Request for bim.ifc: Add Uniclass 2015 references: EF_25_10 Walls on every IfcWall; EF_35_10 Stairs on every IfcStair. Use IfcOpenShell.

First a look at what the model holds.

```python
import ifcopenshell

model = ifcopenshell.open("bim.ifc")
print(model.schema)
print("classifications:", [c.Name for c in model.by_type("IfcClassification")])
for ifc_class in ("IfcDoor", "IfcRoof", "IfcStair", "IfcWall", "IfcWindow"):
    print(ifc_class, len(model.by_type(ifc_class)))
```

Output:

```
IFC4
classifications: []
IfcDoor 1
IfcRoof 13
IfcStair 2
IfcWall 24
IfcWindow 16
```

```python
import ifcopenshell
import ifcopenshell.api.classification

model = ifcopenshell.open("bim.ifc")

system = ifcopenshell.api.classification.add_classification(model, classification="Uniclass 2015")

codes = {
    "IfcWall": ("EF_25_10", "Walls"),
    "IfcStair": ("EF_35_10", "Stairs"),
}
for ifc_class, (code, name) in codes.items():
    products = model.by_type(ifc_class)
    ifcopenshell.api.classification.add_reference(
        model, products=products, classification=system, identification=code, name=name
    )
    print(code, len(products))

model.write("bim_rev.ifc")
```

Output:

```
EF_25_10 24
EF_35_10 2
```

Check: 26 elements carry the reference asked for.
